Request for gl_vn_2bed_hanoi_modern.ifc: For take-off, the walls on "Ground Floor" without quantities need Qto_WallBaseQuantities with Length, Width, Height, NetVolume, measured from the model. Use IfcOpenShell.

First a look at what the model holds.

```python
import ifcopenshell
import ifcopenshell.util.element
import ifcopenshell.util.unit

model = ifcopenshell.open("gl_vn_2bed_hanoi_modern.ifc")
print(model.schema)
for unit_type in ("LENGTHUNIT", "AREAUNIT", "VOLUMEUNIT"):
    print(unit_type, ifcopenshell.util.unit.calculate_unit_scale(model, unit_type))
storey = next(s for s in model.by_type("IfcBuildingStorey") if s.Name == "Ground Floor")
walls = [e for e in ifcopenshell.util.element.get_decomposition(storey) if e.is_a("IfcWall")]
for e in sorted(walls, key=lambda e: e.id()):
    print(e.id(), e.is_a(), e.Name, list(ifcopenshell.util.element.get_psets(e, qtos_only=True)), sep=" | ")
```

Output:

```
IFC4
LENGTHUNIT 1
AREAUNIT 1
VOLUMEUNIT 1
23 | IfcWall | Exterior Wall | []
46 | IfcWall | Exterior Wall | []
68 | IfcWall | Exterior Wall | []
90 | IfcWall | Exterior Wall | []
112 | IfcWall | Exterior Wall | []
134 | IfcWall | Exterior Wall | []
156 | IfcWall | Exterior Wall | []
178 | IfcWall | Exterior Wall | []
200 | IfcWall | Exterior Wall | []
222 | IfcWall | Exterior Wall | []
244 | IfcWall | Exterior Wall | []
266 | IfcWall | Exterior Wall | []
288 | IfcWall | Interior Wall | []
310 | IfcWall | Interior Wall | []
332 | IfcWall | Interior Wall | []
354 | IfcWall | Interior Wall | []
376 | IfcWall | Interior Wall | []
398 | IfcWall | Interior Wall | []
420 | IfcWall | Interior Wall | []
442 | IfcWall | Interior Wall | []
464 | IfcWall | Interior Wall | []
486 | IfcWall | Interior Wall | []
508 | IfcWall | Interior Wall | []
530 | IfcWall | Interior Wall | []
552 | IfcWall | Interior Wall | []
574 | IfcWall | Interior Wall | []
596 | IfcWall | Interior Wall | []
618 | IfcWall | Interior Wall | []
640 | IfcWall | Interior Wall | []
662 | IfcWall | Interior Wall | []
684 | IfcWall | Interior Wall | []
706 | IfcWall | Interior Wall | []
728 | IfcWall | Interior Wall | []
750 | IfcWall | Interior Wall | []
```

```python
import ifcopenshell
import ifcopenshell.api.pset
import ifcopenshell.geom
import ifcopenshell.util.element
import ifcopenshell.util.shape
import ifcopenshell.util.unit

model = ifcopenshell.open("gl_vn_2bed_hanoi_modern.ifc")
unit_scale = ifcopenshell.util.unit.calculate_unit_scale(model)
volume_scale = ifcopenshell.util.unit.calculate_unit_scale(model, "VOLUMEUNIT")
settings = ifcopenshell.geom.settings()

storey = next(s for s in model.by_type("IfcBuildingStorey") if s.Name == "Ground Floor")
walls = [e for e in ifcopenshell.util.element.get_decomposition(storey) if e.is_a("IfcWall")]

for e in sorted(walls, key=lambda e: e.id()):
    if ifcopenshell.util.element.get_psets(e, qtos_only=True, should_inherit=False):
        continue
    # Geometry comes back in metres, in the element's own axes.
    shape = ifcopenshell.geom.create_shape(settings, e)
    values = {
        "Length": ifcopenshell.util.shape.get_x(shape.geometry) / unit_scale,
        "Width": ifcopenshell.util.shape.get_y(shape.geometry) / unit_scale,
        "Height": ifcopenshell.util.shape.get_z(shape.geometry) / unit_scale,
        "NetVolume": ifcopenshell.util.shape.get_volume(shape.geometry) / volume_scale,
    }
    qto = ifcopenshell.api.pset.add_qto(model, product=e, name="Qto_WallBaseQuantities")
    ifcopenshell.api.pset.edit_qto(model, qto=qto, properties=values)
    print(e.id(), {k: round(v, 3) for k, v in values.items()})

model.write("gl_vn_2bed_hanoi_modern_rev.ifc")
```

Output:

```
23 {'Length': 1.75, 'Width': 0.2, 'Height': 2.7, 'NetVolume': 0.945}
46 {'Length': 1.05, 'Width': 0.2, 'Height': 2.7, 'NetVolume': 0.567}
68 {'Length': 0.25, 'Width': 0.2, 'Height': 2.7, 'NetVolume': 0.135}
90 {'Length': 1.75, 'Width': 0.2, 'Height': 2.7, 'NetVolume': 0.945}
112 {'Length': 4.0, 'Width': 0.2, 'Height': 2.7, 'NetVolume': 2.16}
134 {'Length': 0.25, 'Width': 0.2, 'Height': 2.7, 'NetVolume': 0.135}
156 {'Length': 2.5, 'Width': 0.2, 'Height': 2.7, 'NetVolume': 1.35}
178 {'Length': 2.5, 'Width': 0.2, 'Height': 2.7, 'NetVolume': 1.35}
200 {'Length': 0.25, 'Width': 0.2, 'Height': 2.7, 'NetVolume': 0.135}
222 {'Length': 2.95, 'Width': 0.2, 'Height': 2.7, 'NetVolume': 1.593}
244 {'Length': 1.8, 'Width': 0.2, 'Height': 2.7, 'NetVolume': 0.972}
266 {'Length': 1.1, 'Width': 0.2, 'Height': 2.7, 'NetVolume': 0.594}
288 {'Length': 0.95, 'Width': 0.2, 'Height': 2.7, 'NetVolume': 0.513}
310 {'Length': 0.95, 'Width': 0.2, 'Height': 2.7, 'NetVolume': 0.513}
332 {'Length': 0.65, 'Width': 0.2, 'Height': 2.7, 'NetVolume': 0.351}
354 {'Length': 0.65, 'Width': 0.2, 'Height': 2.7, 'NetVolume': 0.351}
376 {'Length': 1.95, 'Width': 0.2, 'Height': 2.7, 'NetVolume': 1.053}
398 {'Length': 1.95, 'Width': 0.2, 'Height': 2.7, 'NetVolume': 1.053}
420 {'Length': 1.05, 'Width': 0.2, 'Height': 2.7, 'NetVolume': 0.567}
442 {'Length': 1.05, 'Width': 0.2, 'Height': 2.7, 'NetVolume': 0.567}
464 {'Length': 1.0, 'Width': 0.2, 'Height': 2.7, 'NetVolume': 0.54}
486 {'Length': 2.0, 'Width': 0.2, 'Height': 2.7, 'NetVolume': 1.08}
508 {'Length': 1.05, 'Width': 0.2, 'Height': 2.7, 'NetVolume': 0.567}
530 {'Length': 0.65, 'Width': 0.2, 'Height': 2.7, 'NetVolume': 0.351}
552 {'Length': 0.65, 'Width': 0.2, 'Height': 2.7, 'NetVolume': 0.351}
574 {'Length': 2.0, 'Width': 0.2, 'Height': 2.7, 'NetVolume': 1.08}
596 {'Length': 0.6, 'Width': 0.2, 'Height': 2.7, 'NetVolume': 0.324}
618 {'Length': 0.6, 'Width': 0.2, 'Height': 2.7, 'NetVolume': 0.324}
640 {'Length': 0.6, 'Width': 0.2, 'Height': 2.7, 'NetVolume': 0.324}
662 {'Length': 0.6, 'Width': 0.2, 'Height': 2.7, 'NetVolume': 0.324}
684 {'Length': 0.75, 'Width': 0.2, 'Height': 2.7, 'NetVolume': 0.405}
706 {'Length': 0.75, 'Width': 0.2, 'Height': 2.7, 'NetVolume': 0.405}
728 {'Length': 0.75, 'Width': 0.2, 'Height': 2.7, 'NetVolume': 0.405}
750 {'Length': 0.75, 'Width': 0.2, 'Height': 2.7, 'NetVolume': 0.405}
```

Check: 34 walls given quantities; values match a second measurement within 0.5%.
